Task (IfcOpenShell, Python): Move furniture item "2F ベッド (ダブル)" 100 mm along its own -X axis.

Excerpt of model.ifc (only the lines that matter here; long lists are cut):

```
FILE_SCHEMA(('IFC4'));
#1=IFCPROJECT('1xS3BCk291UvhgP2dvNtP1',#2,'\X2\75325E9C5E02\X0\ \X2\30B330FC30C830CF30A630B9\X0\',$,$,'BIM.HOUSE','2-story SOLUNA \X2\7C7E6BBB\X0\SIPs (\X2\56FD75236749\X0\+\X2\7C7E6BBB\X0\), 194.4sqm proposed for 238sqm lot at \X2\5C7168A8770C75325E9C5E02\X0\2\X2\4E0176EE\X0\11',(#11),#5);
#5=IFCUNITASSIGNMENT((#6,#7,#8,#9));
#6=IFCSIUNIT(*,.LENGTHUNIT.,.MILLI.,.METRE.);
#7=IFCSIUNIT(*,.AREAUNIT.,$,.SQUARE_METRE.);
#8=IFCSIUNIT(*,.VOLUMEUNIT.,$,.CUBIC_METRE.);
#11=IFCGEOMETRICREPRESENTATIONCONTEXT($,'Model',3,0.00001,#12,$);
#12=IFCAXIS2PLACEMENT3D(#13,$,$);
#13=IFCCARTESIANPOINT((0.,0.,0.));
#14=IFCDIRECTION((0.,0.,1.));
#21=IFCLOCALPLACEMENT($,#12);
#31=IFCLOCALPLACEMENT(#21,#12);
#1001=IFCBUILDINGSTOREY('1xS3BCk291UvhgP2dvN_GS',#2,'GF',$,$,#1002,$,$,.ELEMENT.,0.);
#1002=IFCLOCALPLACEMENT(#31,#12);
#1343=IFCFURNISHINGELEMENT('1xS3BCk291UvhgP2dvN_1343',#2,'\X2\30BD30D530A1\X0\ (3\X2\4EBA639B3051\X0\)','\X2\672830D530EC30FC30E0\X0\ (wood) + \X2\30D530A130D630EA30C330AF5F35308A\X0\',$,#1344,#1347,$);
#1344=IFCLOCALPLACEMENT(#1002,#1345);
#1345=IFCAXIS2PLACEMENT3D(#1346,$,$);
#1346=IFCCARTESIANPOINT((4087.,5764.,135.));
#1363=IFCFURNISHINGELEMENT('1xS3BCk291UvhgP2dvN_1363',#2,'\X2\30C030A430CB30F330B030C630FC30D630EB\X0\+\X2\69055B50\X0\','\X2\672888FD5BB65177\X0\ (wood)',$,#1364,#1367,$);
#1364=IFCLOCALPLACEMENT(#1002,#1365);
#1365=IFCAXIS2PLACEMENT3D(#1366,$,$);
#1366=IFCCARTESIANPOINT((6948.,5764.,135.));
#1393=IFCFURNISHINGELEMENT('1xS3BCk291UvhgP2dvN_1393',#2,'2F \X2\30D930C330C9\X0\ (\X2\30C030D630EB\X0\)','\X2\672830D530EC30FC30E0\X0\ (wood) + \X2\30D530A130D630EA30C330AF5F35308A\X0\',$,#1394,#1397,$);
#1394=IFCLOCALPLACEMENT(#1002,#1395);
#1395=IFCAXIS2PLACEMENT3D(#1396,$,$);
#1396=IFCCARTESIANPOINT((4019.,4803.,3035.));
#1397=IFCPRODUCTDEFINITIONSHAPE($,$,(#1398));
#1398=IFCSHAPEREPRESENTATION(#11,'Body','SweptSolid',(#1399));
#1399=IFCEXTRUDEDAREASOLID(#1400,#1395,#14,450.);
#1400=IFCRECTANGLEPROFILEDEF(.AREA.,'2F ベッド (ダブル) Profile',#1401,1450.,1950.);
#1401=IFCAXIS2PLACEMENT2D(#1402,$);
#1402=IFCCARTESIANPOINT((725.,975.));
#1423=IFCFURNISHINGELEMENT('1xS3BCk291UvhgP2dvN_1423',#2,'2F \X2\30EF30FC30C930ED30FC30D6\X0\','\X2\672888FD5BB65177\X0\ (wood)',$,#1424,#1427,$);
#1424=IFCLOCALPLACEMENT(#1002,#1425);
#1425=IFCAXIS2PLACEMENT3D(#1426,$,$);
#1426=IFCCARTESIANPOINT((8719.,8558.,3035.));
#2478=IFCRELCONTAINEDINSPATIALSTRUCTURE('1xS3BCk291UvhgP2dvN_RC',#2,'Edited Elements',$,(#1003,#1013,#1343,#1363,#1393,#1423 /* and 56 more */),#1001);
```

```python
import ifcopenshell
import ifcopenshell.api.geometry
import ifcopenshell.util.placement
import ifcopenshell.util.unit

model = ifcopenshell.open("model.ifc")
unit_scale = ifcopenshell.util.unit.calculate_unit_scale(model)

item = model.by_id(1393)
matrix = ifcopenshell.util.placement.get_local_placement(item.ObjectPlacement)
matrix[:3, 3] -= matrix[:3, 0] * 0.1 / unit_scale
ifcopenshell.api.geometry.edit_object_placement(model, product=item, matrix=matrix, is_si=False)

print(ifcopenshell.util.placement.get_local_placement(item.ObjectPlacement).round(3) + 0.0)

model.write("model_rev.ifc")
```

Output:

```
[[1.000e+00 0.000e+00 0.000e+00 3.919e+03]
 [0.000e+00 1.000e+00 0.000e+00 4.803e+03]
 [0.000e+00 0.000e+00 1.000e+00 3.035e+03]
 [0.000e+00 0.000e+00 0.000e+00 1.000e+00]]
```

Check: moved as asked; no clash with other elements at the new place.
